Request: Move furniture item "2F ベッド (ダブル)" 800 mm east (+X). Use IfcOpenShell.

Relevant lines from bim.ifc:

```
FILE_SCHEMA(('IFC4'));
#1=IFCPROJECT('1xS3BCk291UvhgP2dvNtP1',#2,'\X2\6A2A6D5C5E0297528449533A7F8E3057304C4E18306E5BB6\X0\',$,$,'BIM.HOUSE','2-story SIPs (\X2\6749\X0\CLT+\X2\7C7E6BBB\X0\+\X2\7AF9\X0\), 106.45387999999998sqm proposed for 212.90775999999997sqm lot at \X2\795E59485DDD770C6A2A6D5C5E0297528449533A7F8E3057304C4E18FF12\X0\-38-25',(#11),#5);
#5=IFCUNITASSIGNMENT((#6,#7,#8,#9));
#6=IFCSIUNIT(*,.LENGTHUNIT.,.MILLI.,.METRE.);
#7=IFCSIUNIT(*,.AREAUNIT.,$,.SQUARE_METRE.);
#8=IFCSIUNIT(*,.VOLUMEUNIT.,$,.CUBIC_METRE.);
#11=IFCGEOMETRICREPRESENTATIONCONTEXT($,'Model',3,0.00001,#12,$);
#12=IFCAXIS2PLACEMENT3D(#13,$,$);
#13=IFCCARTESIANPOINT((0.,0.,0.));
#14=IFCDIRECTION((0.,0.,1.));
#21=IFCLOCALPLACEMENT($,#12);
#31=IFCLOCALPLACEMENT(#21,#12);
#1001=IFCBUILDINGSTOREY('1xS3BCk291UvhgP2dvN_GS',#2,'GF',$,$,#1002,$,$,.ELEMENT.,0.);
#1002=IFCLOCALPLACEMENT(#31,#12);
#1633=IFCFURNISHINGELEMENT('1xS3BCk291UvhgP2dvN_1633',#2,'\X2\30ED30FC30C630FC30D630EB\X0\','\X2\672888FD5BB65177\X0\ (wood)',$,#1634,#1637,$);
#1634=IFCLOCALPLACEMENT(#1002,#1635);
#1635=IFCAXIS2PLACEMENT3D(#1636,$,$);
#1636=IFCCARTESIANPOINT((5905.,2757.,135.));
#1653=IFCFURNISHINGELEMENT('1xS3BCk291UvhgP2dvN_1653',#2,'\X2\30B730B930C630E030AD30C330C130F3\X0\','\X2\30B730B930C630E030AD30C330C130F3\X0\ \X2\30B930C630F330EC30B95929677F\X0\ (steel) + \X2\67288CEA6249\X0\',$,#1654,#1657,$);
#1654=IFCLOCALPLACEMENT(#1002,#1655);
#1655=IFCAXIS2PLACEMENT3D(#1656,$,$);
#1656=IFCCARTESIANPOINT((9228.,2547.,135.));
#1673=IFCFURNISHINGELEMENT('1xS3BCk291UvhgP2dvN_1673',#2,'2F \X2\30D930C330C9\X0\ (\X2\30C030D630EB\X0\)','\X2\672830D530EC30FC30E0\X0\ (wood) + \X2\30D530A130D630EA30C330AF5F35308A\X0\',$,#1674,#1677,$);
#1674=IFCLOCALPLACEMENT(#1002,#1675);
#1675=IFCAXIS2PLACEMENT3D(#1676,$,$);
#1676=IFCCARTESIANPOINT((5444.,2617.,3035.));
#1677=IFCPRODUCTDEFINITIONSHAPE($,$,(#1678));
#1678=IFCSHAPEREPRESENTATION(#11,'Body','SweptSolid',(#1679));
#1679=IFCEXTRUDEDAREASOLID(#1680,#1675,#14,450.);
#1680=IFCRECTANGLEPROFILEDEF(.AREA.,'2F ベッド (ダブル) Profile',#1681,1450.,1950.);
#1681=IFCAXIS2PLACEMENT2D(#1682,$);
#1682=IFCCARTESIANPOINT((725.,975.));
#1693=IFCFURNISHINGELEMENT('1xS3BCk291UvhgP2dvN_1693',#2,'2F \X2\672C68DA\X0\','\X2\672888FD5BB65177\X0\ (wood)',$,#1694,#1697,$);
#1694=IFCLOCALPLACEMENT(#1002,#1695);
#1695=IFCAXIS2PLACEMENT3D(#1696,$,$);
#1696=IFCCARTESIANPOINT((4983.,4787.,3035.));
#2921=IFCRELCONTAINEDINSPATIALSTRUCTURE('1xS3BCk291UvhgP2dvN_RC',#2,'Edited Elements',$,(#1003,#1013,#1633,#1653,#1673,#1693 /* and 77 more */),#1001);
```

```python
import ifcopenshell
import ifcopenshell.api.geometry
import ifcopenshell.util.placement

model = ifcopenshell.open("bim.ifc")

item = model.by_guid("1xS3BCk291UvhgP2dvN_1673")
matrix = ifcopenshell.util.placement.get_local_placement(item.ObjectPlacement)
matrix[0, 3] += 800.0
ifcopenshell.api.geometry.edit_object_placement(model, product=item, matrix=matrix, is_si=False)

print(ifcopenshell.util.placement.get_local_placement(item.ObjectPlacement).round(3) + 0.0)

model.write("bim_v2.ifc")
```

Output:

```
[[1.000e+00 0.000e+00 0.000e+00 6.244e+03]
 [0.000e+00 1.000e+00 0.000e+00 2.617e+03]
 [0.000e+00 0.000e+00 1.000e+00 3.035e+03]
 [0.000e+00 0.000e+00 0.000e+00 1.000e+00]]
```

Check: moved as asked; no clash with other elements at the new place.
